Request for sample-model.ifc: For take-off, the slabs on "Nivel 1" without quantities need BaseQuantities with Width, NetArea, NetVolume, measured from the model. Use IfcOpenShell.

First a look at what the model holds.

```python
import ifcopenshell
import ifcopenshell.util.element
import ifcopenshell.util.unit

model = ifcopenshell.open("sample-model.ifc")
print(model.schema)
for unit_type in ("LENGTHUNIT", "AREAUNIT", "VOLUMEUNIT"):
    print(unit_type, ifcopenshell.util.unit.calculate_unit_scale(model, unit_type))
storey = next(s for s in model.by_type("IfcBuildingStorey") if s.Name == "Nivel 1")
slabs = [e for e in ifcopenshell.util.element.get_decomposition(storey) if e.is_a("IfcSlab")]
for e in sorted(slabs, key=lambda e: e.id()):
    print(e.id(), e.is_a(), e.Name, list(ifcopenshell.util.element.get_psets(e, qtos_only=True)), sep=" | ")
```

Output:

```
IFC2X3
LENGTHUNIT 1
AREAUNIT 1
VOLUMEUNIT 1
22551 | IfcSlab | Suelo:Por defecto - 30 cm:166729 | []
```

```python
import ifcopenshell
import ifcopenshell.api.pset
import ifcopenshell.geom
import ifcopenshell.util.element
import ifcopenshell.util.shape
import ifcopenshell.util.unit

model = ifcopenshell.open("sample-model.ifc")
unit_scale = ifcopenshell.util.unit.calculate_unit_scale(model)
area_scale = ifcopenshell.util.unit.calculate_unit_scale(model, "AREAUNIT")
volume_scale = ifcopenshell.util.unit.calculate_unit_scale(model, "VOLUMEUNIT")
settings = ifcopenshell.geom.settings()

storey = next(s for s in model.by_type("IfcBuildingStorey") if s.Name == "Nivel 1")
slabs = [e for e in ifcopenshell.util.element.get_decomposition(storey) if e.is_a("IfcSlab")]

for e in sorted(slabs, key=lambda e: e.id()):
    if ifcopenshell.util.element.get_psets(e, qtos_only=True, should_inherit=False):
        continue
    # Geometry comes back in metres, in the element's own axes.
    shape = ifcopenshell.geom.create_shape(settings, e)
    values = {
        "Width": ifcopenshell.util.shape.get_z(shape.geometry) / unit_scale,
        "NetArea": ifcopenshell.util.shape.get_footprint_area(shape.geometry) / area_scale,
        "NetVolume": ifcopenshell.util.shape.get_volume(shape.geometry) / volume_scale,
    }
    qto = ifcopenshell.api.pset.add_qto(model, product=e, name="BaseQuantities")
    ifcopenshell.api.pset.edit_qto(model, qto=qto, properties=values)
    print(e.id(), {k: round(v, 3) for k, v in values.items()})

model.write("sample-model_rev.ifc")
```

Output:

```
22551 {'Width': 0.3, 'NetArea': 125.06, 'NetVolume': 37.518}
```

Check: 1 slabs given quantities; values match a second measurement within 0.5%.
